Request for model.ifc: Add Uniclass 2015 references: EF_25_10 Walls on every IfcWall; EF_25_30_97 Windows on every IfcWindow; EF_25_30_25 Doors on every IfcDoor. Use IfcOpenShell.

First a look at what the model holds.

```python
import ifcopenshell

model = ifcopenshell.open("model.ifc")
print(model.schema)
print("classifications:", [c.Name for c in model.by_type("IfcClassification")])
for ifc_class in ("IfcDoor", "IfcRoof", "IfcStair", "IfcWall", "IfcWindow"):
    print(ifc_class, len(model.by_type(ifc_class)))
```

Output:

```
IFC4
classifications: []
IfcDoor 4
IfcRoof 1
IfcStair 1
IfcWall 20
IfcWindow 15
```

```python
import ifcopenshell
import ifcopenshell.api.classification

model = ifcopenshell.open("model.ifc")

system = ifcopenshell.api.classification.add_classification(model, classification="Uniclass 2015")

codes = {
    "IfcWall": ("EF_25_10", "Walls"),
    "IfcWindow": ("EF_25_30_97", "Windows"),
    "IfcDoor": ("EF_25_30_25", "Doors"),
}
for ifc_class, (code, name) in codes.items():
    products = model.by_type(ifc_class)
    ifcopenshell.api.classification.add_reference(
        model, products=products, classification=system, identification=code, name=name
    )
    print(code, len(products))

model.write("model_rev.ifc")
```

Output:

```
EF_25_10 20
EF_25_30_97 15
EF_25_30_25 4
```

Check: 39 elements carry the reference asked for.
